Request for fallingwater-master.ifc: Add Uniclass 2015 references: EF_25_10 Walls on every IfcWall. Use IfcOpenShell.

First a look at what the model holds.

```python
import ifcopenshell

model = ifcopenshell.open("fallingwater-master.ifc")
print(model.schema)
print("classifications:", [c.Name for c in model.by_type("IfcClassification")])
for ifc_class in ("IfcDoor", "IfcRoof", "IfcStair", "IfcWall", "IfcWindow"):
    print(ifc_class, len(model.by_type(ifc_class)))
```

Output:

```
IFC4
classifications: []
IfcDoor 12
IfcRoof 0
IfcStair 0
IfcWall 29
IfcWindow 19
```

```python
import ifcopenshell
import ifcopenshell.api.classification

model = ifcopenshell.open("fallingwater-master.ifc")

system = ifcopenshell.api.classification.add_classification(model, classification="Uniclass 2015")

codes = {
    "IfcWall": ("EF_25_10", "Walls"),
}
for ifc_class, (code, name) in codes.items():
    products = model.by_type(ifc_class)
    ifcopenshell.api.classification.add_reference(
        model, products=products, classification=system, identification=code, name=name
    )
    print(code, len(products))

model.write("fallingwater-master_updated.ifc")
```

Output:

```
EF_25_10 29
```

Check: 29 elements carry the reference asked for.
